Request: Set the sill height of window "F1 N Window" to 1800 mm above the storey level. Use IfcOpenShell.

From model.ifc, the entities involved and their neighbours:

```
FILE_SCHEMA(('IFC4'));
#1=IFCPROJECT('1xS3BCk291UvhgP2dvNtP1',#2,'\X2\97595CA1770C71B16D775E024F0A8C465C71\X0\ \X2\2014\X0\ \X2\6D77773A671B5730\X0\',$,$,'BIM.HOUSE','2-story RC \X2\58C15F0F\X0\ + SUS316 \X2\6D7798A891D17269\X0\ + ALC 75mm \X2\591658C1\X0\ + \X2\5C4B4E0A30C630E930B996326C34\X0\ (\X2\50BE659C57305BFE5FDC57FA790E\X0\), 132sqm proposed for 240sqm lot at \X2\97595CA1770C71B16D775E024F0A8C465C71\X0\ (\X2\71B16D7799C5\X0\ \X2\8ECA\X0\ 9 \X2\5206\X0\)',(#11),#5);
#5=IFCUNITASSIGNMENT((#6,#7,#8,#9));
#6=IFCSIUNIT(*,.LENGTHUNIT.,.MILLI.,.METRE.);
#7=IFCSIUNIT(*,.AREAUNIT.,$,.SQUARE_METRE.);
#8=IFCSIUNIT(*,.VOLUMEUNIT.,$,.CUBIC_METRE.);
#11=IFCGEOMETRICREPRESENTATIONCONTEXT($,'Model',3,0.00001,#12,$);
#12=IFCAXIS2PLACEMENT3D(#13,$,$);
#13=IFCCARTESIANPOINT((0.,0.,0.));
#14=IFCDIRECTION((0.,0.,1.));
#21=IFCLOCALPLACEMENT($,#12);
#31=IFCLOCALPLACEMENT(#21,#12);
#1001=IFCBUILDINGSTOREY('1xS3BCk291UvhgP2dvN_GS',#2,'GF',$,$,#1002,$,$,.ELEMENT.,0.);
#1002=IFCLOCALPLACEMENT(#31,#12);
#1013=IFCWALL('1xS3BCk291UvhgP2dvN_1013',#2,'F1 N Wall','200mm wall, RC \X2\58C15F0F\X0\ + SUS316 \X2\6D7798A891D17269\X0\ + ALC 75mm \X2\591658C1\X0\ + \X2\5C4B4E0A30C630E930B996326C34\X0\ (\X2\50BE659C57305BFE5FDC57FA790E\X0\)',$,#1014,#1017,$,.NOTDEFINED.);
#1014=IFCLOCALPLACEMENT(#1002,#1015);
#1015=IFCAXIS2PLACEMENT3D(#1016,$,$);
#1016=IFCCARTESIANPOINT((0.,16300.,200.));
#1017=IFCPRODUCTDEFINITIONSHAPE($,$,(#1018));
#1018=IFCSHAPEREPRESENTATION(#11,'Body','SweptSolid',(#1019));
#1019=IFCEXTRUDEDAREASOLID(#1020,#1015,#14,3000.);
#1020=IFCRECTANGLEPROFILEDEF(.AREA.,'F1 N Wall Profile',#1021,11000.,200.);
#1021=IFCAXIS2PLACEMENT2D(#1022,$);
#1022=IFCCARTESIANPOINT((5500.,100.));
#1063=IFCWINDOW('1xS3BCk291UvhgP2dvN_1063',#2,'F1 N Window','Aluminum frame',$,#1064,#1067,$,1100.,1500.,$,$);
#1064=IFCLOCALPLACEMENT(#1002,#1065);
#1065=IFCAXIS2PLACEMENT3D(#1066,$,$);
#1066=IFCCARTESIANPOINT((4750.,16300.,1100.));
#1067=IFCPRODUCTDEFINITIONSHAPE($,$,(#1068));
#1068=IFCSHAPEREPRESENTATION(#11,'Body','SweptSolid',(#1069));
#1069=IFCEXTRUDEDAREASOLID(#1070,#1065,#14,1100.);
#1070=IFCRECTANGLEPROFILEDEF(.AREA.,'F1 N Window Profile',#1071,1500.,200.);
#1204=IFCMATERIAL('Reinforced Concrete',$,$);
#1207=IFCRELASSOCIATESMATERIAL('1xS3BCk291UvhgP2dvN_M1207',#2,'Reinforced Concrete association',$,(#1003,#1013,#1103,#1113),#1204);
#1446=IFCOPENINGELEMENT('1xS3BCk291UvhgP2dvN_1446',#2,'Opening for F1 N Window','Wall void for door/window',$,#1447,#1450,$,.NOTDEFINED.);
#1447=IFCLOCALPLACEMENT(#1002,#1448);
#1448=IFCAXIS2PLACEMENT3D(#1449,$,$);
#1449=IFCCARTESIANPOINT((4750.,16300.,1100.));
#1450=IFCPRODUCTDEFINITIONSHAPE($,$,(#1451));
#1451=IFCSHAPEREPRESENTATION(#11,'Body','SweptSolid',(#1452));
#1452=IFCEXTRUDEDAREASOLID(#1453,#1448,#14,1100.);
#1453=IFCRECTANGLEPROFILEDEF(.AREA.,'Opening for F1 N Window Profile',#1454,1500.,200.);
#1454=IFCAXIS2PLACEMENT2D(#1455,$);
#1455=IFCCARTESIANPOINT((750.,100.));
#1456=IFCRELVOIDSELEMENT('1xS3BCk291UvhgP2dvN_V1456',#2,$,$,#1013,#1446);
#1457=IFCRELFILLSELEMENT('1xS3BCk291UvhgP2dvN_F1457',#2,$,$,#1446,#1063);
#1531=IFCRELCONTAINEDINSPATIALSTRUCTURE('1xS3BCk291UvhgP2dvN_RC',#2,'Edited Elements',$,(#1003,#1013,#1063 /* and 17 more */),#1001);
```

```python
import numpy as np
import ifcopenshell
import ifcopenshell.api.geometry
import ifcopenshell.geom
import ifcopenshell.util.element
import ifcopenshell.util.placement
import ifcopenshell.util.shape
import ifcopenshell.util.unit

model = ifcopenshell.open("model.ifc")
unit_scale = ifcopenshell.util.unit.calculate_unit_scale(model)

window = model.by_guid("1xS3BCk291UvhgP2dvN_1063")
opening = window.FillsVoids[0].RelatingOpeningElement
storey = ifcopenshell.util.element.get_container(window, ifc_class="IfcBuildingStorey")
level = ifcopenshell.util.placement.get_local_placement(storey.ObjectPlacement)[2, 3]

# The opening's origin need not be at the sill, so measure its lowest point.
shape = ifcopenshell.geom.create_shape(ifcopenshell.geom.settings(), opening)
bottom = ifcopenshell.util.shape.get_shape_bottom_elevation(shape, shape.geometry) / unit_scale
dz = level + 1800.0 - bottom

shift = np.array([0.0, 0.0, dz])
# The window is not placed relative to its opening, so move both.
for product in (opening, window):
    matrix = ifcopenshell.util.placement.get_local_placement(product.ObjectPlacement)
    matrix[:3, 3] += shift
    ifcopenshell.api.geometry.edit_object_placement(model, product=product, matrix=matrix, is_si=False)

print(f"moved by {dz * unit_scale:+.3f} m")

model.write("model-out.ifc")
```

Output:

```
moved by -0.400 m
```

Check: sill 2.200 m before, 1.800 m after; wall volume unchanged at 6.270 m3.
